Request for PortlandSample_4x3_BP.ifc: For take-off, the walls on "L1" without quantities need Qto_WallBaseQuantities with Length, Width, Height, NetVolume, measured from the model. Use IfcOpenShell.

First a look at what the model holds.

```python
import ifcopenshell
import ifcopenshell.util.element
import ifcopenshell.util.unit

model = ifcopenshell.open("PortlandSample_4x3_BP.ifc")
print(model.schema)
for unit_type in ("LENGTHUNIT", "AREAUNIT", "VOLUMEUNIT"):
    print(unit_type, ifcopenshell.util.unit.calculate_unit_scale(model, unit_type))
storey = next(s for s in model.by_type("IfcBuildingStorey") if s.Name == "L1")
walls = [e for e in ifcopenshell.util.element.get_decomposition(storey) if e.is_a("IfcWall")]
for e in sorted(walls, key=lambda e: e.id()):
    print(e.id(), e.is_a(), e.Name, list(ifcopenshell.util.element.get_psets(e, qtos_only=True)), sep=" | ")
```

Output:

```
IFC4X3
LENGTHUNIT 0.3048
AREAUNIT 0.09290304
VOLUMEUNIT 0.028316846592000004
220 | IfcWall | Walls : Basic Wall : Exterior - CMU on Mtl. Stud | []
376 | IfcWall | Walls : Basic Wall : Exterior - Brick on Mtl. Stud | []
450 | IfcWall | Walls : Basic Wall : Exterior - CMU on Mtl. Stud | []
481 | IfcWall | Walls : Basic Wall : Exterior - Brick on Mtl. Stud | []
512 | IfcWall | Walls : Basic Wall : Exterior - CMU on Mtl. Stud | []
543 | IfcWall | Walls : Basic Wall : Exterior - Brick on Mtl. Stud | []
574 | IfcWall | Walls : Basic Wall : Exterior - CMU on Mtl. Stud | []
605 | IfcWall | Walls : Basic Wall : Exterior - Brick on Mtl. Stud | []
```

```python
import ifcopenshell
import ifcopenshell.api.pset
import ifcopenshell.geom
import ifcopenshell.util.element
import ifcopenshell.util.shape
import ifcopenshell.util.unit

model = ifcopenshell.open("PortlandSample_4x3_BP.ifc")
unit_scale = ifcopenshell.util.unit.calculate_unit_scale(model)
volume_scale = ifcopenshell.util.unit.calculate_unit_scale(model, "VOLUMEUNIT")
settings = ifcopenshell.geom.settings()

storey = next(s for s in model.by_type("IfcBuildingStorey") if s.Name == "L1")
walls = [e for e in ifcopenshell.util.element.get_decomposition(storey) if e.is_a("IfcWall")]

for e in sorted(walls, key=lambda e: e.id()):
    if ifcopenshell.util.element.get_psets(e, qtos_only=True, should_inherit=False):
        continue
    # Geometry comes back in metres, in the element's own axes.
    shape = ifcopenshell.geom.create_shape(settings, e)
    values = {
        "Length": ifcopenshell.util.shape.get_x(shape.geometry) / unit_scale,
        "Width": ifcopenshell.util.shape.get_y(shape.geometry) / unit_scale,
        "Height": ifcopenshell.util.shape.get_z(shape.geometry) / unit_scale,
        "NetVolume": ifcopenshell.util.shape.get_volume(shape.geometry) / volume_scale,
    }
    qto = ifcopenshell.api.pset.add_qto(model, product=e, name="Qto_WallBaseQuantities")
    ifcopenshell.api.pset.edit_qto(model, qto=qto, properties=values)
    print(e.id(), {k: round(v, 3) for k, v in values.items()})

model.write("PortlandSample_4x3_BP-out.ifc")
```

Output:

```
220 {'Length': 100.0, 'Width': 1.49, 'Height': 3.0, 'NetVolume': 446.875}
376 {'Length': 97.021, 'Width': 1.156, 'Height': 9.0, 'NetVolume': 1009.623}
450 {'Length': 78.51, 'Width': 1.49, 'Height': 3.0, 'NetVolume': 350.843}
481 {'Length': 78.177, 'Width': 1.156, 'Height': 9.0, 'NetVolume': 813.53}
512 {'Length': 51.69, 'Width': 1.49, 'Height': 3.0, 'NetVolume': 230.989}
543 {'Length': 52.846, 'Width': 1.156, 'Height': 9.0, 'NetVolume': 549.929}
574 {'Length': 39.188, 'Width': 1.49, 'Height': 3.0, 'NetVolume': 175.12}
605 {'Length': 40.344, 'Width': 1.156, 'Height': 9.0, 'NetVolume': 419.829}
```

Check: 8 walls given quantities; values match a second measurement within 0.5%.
